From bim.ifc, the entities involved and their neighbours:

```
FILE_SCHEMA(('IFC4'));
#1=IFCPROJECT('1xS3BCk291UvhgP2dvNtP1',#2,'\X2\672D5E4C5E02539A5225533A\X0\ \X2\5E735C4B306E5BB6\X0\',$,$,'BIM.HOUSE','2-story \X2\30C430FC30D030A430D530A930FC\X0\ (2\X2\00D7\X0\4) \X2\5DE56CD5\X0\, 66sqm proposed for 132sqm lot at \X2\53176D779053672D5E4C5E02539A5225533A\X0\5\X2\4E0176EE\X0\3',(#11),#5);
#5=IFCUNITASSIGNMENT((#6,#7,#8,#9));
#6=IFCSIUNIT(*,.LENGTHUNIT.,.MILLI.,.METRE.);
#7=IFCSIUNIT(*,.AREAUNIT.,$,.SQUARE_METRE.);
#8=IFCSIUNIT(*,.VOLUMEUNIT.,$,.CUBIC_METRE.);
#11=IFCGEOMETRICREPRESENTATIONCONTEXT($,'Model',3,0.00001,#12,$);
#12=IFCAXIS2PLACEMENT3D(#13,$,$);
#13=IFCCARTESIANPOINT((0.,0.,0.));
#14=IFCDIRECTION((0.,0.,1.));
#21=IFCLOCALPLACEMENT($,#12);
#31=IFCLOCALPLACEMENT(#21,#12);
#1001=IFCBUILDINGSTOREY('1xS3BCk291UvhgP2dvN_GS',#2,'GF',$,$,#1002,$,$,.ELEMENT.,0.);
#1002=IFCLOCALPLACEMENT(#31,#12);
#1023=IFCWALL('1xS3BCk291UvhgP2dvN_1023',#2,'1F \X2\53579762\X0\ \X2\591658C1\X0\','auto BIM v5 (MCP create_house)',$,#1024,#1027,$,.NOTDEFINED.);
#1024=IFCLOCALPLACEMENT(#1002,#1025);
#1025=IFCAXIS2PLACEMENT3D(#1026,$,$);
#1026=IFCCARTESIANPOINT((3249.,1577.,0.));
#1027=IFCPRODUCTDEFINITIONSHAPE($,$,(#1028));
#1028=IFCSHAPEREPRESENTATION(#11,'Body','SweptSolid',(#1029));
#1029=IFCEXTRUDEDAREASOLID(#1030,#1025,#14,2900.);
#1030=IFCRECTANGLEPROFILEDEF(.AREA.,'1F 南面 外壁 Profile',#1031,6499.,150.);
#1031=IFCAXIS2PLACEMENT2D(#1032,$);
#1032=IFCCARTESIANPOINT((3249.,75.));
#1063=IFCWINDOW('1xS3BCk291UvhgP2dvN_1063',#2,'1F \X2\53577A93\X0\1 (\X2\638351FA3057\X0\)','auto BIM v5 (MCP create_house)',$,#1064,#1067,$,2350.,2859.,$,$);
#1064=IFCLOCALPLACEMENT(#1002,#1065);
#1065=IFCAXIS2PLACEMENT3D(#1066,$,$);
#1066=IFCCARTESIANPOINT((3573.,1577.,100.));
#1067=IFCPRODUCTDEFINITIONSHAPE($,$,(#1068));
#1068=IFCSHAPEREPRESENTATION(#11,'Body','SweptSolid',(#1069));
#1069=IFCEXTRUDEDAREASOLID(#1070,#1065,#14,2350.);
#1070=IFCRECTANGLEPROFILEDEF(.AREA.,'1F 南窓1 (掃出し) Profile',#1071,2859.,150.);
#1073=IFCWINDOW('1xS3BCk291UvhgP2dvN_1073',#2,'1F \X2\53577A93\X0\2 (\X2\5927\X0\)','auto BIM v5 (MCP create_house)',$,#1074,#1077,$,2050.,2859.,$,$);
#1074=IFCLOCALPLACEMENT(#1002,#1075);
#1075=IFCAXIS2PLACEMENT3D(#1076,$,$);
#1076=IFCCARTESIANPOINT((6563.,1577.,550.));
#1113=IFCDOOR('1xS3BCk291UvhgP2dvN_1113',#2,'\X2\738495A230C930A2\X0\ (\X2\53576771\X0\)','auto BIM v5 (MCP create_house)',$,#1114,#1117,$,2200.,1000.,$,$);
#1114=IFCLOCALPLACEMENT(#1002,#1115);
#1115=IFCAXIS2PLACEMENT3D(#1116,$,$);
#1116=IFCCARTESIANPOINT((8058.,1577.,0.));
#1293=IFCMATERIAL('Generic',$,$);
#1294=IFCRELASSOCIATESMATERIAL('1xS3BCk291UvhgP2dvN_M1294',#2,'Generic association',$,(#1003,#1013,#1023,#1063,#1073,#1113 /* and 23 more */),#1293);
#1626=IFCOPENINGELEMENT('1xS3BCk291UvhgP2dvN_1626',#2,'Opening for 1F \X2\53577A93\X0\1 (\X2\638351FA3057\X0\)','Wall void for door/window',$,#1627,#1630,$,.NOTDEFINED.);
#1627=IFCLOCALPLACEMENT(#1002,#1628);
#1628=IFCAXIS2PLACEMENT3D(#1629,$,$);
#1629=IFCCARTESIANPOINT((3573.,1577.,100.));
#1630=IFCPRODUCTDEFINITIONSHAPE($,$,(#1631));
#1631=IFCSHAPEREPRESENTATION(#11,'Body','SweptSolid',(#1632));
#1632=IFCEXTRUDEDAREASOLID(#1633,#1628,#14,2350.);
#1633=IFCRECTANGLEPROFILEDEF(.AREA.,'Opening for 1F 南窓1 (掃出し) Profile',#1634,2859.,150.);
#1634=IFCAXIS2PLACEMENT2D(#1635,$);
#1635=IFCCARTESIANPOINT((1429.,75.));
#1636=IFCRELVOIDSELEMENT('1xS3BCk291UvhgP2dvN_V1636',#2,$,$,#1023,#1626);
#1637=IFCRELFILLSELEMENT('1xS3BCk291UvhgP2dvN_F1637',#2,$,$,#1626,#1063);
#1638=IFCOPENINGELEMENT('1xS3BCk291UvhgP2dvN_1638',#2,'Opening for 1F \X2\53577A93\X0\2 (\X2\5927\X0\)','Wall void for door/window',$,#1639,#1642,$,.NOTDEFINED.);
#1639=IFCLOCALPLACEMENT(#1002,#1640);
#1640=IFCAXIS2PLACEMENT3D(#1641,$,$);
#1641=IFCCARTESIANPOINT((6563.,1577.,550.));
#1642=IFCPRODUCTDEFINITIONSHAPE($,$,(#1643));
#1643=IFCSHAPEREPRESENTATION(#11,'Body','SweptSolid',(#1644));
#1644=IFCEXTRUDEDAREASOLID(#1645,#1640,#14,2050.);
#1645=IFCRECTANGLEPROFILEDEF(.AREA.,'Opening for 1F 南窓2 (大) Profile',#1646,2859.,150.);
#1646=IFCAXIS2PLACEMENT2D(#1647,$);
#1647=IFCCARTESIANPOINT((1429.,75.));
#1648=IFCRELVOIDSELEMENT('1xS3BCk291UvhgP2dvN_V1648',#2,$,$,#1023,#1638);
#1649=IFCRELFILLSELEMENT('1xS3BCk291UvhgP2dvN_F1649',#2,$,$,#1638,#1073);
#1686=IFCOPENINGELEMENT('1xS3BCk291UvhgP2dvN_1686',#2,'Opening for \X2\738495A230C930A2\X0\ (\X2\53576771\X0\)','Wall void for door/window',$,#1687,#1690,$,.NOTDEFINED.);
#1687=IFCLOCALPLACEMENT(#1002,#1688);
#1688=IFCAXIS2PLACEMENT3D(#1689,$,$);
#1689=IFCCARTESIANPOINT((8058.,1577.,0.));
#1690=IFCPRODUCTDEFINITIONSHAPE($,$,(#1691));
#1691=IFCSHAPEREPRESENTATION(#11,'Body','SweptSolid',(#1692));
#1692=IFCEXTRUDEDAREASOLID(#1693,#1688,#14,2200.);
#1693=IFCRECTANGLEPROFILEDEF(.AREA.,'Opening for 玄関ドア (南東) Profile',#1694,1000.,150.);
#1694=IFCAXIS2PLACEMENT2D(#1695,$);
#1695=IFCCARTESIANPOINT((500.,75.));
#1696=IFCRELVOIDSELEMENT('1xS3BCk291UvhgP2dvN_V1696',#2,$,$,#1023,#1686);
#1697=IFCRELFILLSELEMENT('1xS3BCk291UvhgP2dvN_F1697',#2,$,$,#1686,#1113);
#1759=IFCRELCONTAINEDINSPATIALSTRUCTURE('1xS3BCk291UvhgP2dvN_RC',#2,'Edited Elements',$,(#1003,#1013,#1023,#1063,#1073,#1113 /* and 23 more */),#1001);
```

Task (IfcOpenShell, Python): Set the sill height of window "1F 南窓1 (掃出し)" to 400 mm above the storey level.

```python
import numpy as np
import ifcopenshell
import ifcopenshell.api.geometry
import ifcopenshell.geom
import ifcopenshell.util.element
import ifcopenshell.util.placement
import ifcopenshell.util.shape
import ifcopenshell.util.unit

model = ifcopenshell.open("bim.ifc")
unit_scale = ifcopenshell.util.unit.calculate_unit_scale(model)

window = model.by_id(1063)
opening = window.FillsVoids[0].RelatingOpeningElement
storey = ifcopenshell.util.element.get_container(window, ifc_class="IfcBuildingStorey")
level = ifcopenshell.util.placement.get_local_placement(storey.ObjectPlacement)[2, 3]

# The opening's origin need not be at the sill, so measure its lowest point.
shape = ifcopenshell.geom.create_shape(ifcopenshell.geom.settings(), opening)
bottom = ifcopenshell.util.shape.get_shape_bottom_elevation(shape, shape.geometry) / unit_scale
dz = level + 0.4 / unit_scale - bottom

shift = np.array([0.0, 0.0, dz])
# The window is not placed relative to its opening, so move both.
for product in (opening, window):
    matrix = ifcopenshell.util.placement.get_local_placement(product.ObjectPlacement)
    matrix[:3, 3] += shift
    ifcopenshell.api.geometry.edit_object_placement(model, product=product, matrix=matrix, is_si=False)

print(f"moved by {dz * unit_scale:+.3f} m")

model.write("bim_updated.ifc")
```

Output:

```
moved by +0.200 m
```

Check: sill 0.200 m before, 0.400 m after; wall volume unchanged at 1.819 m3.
